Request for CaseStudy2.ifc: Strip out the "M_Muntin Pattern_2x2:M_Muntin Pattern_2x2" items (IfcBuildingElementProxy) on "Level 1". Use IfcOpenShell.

First a look at what the model holds.

```python
import ifcopenshell
import ifcopenshell.util.element

model = ifcopenshell.open("CaseStudy2.ifc")
print(model.schema)
storey = next(s for s in model.by_type("IfcBuildingStorey") if s.Name == "Level 1")
proxies = [e for e in ifcopenshell.util.element.get_decomposition(storey) if e.is_a("IfcBuildingElementProxy")]
seen = {}
for e in proxies:
    element_type = ifcopenshell.util.element.get_type(e)
    name = element_type.Name if element_type not in (None, e) else None
    seen[name] = seen.get(name, 0) + 1
for name, count in sorted(seen.items(), key=str):
    print(count, "x", name)
```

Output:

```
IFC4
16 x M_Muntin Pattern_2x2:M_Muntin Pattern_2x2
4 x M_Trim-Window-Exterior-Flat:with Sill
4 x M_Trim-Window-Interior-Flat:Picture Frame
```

```python
import ifcopenshell
import ifcopenshell.api.root
import ifcopenshell.util.element

model = ifcopenshell.open("CaseStudy2.ifc")

storey = next(s for s in model.by_type("IfcBuildingStorey") if s.Name == "Level 1")
proxies = [e for e in ifcopenshell.util.element.get_decomposition(storey) if e.is_a("IfcBuildingElementProxy")]
targets = [e for e in proxies if (t := ifcopenshell.util.element.get_type(e)) not in (None, e) and t.Name == "M_Muntin Pattern_2x2:M_Muntin Pattern_2x2"]

for e in targets:
    ifcopenshell.api.root.remove_product(model, product=e)
print(len(targets), "removed")

model.write("CaseStudy2_edited.ifc")
```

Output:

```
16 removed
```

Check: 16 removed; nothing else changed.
